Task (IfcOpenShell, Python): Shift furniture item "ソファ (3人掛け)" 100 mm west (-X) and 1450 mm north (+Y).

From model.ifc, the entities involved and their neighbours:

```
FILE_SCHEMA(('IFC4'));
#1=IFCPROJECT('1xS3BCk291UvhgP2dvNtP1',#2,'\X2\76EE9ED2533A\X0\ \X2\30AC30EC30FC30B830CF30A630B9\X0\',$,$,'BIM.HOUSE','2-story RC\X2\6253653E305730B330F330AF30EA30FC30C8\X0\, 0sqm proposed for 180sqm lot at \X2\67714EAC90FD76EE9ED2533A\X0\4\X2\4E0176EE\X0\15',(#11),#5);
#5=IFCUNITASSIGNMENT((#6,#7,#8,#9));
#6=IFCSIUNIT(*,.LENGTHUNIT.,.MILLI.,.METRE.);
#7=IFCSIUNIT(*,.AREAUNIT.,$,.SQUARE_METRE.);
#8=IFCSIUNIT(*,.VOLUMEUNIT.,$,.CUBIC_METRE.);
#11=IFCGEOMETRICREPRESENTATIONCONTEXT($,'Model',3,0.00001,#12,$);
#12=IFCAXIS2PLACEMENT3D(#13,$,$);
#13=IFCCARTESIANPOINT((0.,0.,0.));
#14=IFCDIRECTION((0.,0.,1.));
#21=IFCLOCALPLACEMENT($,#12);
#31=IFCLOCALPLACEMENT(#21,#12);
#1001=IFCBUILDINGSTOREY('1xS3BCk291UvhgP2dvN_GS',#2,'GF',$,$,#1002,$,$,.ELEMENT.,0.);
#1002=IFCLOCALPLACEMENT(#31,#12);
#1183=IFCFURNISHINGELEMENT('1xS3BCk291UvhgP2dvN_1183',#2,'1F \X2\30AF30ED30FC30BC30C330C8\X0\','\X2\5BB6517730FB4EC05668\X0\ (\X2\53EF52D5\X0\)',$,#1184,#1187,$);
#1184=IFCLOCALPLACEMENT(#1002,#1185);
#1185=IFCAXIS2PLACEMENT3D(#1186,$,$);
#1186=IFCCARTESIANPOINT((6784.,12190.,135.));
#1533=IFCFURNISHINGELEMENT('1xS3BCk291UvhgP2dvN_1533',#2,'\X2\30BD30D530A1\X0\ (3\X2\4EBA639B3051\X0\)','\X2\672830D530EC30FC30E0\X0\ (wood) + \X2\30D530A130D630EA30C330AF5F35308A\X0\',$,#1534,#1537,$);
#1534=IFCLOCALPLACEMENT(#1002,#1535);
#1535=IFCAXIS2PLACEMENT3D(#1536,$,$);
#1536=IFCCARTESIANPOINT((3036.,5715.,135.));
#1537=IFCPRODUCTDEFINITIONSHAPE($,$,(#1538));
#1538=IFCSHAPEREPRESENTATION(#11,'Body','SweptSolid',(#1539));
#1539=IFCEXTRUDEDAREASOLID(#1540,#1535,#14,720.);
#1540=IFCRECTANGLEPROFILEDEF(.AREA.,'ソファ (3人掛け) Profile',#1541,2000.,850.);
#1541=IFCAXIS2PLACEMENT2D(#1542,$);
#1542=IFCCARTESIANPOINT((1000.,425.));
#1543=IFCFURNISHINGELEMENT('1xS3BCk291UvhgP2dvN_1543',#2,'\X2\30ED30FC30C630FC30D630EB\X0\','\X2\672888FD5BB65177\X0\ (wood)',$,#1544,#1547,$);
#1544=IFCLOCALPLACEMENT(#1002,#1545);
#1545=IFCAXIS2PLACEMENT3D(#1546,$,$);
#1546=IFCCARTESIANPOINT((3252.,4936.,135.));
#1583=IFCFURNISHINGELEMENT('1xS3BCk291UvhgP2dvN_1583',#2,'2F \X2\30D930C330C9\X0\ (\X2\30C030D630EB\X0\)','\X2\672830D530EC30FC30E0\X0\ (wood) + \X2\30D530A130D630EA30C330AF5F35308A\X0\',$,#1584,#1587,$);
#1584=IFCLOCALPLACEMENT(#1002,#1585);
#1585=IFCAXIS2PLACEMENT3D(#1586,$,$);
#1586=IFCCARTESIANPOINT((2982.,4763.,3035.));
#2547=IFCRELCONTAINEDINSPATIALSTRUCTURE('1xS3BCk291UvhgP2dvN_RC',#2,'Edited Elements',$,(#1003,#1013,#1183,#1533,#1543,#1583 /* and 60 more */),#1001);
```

```python
import ifcopenshell
import ifcopenshell.api.geometry
import ifcopenshell.util.placement
import ifcopenshell.util.unit

model = ifcopenshell.open("model.ifc")
unit_scale = ifcopenshell.util.unit.calculate_unit_scale(model)

item = model.by_guid("1xS3BCk291UvhgP2dvN_1533")
matrix = ifcopenshell.util.placement.get_local_placement(item.ObjectPlacement)
matrix[0, 3] -= 0.1 / unit_scale
matrix[1, 3] += 1.45 / unit_scale
ifcopenshell.api.geometry.edit_object_placement(model, product=item, matrix=matrix, is_si=False)

print(ifcopenshell.util.placement.get_local_placement(item.ObjectPlacement).round(3) + 0.0)

model.write("model-out.ifc")
```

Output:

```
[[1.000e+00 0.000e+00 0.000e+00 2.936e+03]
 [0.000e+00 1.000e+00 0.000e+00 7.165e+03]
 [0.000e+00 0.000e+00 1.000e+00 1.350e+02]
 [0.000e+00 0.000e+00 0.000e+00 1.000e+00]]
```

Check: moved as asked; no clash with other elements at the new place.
